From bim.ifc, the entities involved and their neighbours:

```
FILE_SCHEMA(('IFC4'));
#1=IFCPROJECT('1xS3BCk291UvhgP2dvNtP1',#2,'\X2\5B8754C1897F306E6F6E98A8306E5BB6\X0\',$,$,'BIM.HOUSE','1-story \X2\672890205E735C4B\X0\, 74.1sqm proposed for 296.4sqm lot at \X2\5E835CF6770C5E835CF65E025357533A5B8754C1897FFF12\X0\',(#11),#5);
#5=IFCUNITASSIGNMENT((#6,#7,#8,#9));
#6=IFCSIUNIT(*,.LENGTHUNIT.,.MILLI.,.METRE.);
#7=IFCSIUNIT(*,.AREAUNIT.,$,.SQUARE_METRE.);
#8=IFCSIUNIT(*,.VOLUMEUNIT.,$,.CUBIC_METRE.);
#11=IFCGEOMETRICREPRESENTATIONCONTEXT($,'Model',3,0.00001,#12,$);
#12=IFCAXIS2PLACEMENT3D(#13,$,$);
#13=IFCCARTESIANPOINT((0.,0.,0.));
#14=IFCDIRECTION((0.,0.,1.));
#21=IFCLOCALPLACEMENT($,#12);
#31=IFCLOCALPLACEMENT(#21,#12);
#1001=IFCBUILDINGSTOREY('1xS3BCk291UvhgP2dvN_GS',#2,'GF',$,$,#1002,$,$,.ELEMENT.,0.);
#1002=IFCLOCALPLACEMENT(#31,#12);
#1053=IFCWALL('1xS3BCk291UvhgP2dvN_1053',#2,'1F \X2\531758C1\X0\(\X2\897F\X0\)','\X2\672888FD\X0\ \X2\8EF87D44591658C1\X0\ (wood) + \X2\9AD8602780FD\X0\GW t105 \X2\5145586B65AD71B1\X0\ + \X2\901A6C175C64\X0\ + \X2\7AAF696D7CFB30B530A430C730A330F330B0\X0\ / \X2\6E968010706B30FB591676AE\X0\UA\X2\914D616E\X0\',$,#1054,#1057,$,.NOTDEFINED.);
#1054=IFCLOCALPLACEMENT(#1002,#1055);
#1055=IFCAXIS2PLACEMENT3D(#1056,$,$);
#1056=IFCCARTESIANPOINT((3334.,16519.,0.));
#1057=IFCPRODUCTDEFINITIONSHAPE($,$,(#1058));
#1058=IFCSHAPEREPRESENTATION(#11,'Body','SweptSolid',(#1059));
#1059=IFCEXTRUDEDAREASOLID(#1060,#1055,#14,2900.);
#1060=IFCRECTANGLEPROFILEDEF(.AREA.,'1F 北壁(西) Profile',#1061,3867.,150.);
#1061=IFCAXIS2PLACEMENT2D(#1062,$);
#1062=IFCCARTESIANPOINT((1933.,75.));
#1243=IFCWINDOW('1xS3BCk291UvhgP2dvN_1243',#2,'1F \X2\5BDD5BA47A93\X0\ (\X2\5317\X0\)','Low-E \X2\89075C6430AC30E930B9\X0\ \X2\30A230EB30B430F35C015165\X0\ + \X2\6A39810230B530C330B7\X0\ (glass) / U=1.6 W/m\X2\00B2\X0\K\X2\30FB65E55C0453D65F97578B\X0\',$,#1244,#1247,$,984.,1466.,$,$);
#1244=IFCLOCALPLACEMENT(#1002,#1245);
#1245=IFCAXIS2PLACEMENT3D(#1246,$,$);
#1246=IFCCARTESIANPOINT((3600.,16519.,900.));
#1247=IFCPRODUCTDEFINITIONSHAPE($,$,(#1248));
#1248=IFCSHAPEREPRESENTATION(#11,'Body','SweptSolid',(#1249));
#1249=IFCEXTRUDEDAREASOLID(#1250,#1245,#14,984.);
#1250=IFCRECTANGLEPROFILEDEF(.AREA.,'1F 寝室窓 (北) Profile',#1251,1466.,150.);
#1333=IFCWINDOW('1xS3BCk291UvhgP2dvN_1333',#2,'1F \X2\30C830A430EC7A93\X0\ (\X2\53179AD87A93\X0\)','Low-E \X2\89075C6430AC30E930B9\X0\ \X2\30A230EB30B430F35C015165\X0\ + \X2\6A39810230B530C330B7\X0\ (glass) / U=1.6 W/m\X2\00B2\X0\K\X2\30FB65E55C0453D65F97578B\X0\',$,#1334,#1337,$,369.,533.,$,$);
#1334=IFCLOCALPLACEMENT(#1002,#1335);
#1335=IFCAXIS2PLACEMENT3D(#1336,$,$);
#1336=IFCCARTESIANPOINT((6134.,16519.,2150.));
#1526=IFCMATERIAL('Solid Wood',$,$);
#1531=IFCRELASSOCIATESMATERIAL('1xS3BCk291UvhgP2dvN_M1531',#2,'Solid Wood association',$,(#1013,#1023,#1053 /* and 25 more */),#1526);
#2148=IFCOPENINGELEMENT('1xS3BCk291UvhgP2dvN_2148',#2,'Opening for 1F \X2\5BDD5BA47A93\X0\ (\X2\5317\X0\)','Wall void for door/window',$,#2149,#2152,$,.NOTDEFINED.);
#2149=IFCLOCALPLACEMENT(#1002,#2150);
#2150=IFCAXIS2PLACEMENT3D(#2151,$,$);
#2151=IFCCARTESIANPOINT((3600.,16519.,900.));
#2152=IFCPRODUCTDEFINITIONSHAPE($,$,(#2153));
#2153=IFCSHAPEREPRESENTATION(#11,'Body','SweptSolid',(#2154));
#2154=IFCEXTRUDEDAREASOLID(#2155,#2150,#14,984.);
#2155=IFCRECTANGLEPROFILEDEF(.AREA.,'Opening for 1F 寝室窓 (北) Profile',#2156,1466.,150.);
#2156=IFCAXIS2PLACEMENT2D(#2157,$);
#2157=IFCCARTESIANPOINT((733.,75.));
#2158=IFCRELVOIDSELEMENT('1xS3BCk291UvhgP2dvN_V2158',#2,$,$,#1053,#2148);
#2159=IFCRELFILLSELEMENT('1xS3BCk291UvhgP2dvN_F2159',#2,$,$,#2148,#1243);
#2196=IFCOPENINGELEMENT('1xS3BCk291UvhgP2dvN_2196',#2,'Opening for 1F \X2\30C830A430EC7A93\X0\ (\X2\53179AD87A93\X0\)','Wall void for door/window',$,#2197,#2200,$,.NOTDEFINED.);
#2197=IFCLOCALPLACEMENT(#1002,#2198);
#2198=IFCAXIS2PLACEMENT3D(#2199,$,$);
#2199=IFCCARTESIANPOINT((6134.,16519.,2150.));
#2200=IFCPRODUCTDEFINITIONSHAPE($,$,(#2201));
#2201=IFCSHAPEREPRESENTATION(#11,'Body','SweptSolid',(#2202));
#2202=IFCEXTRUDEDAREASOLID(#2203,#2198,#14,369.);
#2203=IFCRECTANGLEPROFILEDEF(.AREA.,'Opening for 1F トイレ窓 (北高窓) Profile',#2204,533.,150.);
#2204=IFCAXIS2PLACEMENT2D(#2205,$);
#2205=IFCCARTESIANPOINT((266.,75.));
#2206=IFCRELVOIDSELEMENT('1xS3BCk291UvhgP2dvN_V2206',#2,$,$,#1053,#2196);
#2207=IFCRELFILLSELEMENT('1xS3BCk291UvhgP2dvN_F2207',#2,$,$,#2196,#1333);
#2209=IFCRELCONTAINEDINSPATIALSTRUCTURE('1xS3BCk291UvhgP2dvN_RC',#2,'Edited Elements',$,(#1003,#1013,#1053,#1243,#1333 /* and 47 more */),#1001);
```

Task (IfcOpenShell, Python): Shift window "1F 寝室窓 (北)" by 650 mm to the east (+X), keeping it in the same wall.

```python
import ifcopenshell
import ifcopenshell.api.geometry
import ifcopenshell.util.placement
import ifcopenshell.util.unit

model = ifcopenshell.open("bim.ifc")
unit_scale = ifcopenshell.util.unit.calculate_unit_scale(model)

window = model.by_guid("1xS3BCk291UvhgP2dvN_1243")
opening = window.FillsVoids[0].RelatingOpeningElement
wall = opening.VoidsElements[0].RelatingBuildingElement

wall_matrix = ifcopenshell.util.placement.get_local_placement(wall.ObjectPlacement)
shift = wall_matrix[:3, 0] * 0.65 / unit_scale
before = ifcopenshell.util.placement.get_local_placement(window.ObjectPlacement)[:3, 3].copy()

# The window is not placed relative to its opening, so move both.
for product in (opening, window):
    matrix = ifcopenshell.util.placement.get_local_placement(product.ObjectPlacement)
    matrix[:3, 3] += shift
    ifcopenshell.api.geometry.edit_object_placement(model, product=product, matrix=matrix, is_si=False)

after = ifcopenshell.util.placement.get_local_placement(window.ObjectPlacement)[:3, 3]
print("window moved by", (after - before).round(3) + 0.0)

model.write("bim_updated.ifc")
```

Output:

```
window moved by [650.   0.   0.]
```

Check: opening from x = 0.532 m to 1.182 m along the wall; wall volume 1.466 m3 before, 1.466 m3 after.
